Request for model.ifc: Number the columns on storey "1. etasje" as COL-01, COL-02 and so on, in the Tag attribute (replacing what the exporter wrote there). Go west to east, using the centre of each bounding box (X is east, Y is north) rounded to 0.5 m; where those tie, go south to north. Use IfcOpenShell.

First a look at what the model holds.

```python
import ifcopenshell
import ifcopenshell.util.element
import ifcopenshell.util.placement

model = ifcopenshell.open("model.ifc")
print(model.schema)
storey = next(s for s in model.by_type("IfcBuildingStorey") if s.Name == "1. etasje")
columns = [e for e in ifcopenshell.util.element.get_decomposition(storey) if e.is_a("IfcColumn")]
for e in sorted(columns, key=lambda e: e.id()):
    origin = ifcopenshell.util.placement.get_local_placement(e.ObjectPlacement)[:3, 3]
    print(e.id(), e.Tag, e.Name, origin.round(2) + 0.0, sep=" | ")
```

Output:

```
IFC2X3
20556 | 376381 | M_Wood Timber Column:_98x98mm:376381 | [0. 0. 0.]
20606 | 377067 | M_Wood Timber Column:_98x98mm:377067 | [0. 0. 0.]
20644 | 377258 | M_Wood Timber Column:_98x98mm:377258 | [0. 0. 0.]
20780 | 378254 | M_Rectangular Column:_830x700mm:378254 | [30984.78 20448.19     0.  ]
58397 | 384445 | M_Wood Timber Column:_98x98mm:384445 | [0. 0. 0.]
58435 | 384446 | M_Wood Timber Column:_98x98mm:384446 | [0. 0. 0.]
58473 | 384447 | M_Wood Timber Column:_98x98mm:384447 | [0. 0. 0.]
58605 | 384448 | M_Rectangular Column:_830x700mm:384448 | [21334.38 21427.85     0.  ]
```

```python
import ifcopenshell
import ifcopenshell.geom
import ifcopenshell.util.element
import ifcopenshell.util.shape

model = ifcopenshell.open("model.ifc")
settings = ifcopenshell.geom.settings()
settings.set("use-world-coords", True)


def centre(element):
    shape = ifcopenshell.geom.create_shape(settings, element)
    return ifcopenshell.util.shape.get_bbox_centroid(shape.geometry)


storey = next(s for s in model.by_type("IfcBuildingStorey") if s.Name == "1. etasje")
columns = [e for e in ifcopenshell.util.element.get_decomposition(storey) if e.is_a("IfcColumn")]

# Insertion points can sit at a corner or the storey origin, so sort by the geometry (in metres).
centres = {e: centre(e) for e in columns}
columns.sort(key=lambda e: (round(centres[e][0] / 0.5), centres[e][1]))

for i, e in enumerate(columns, start=1):
    number = f"COL-{i:02d}"
    e.Tag = number
    print(e.id(), number)

model.write("model_rev.ifc")
```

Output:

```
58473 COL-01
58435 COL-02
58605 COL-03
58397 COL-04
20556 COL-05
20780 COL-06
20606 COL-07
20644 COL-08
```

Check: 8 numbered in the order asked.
